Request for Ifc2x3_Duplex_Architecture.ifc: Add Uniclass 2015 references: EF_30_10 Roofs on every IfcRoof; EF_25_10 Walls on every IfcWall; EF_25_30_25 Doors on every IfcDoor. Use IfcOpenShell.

First a look at what the model holds.

```python
import ifcopenshell

model = ifcopenshell.open("Ifc2x3_Duplex_Architecture.ifc")
print(model.schema)
print("classifications:", [c.Name for c in model.by_type("IfcClassification")])
for ifc_class in ("IfcDoor", "IfcRoof", "IfcStair", "IfcWall", "IfcWindow"):
    print(ifc_class, len(model.by_type(ifc_class)))
```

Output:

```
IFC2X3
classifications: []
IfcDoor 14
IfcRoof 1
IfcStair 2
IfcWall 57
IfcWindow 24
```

```python
import ifcopenshell
import ifcopenshell.api.classification

model = ifcopenshell.open("Ifc2x3_Duplex_Architecture.ifc")

# IFC2X3 requires Source and Edition and has no link from the project to the system.
system = model.create_entity("IfcClassification", Source="NBS", Edition="2015", Name="Uniclass 2015")

codes = {
    "IfcRoof": ("EF_30_10", "Roofs"),
    "IfcWall": ("EF_25_10", "Walls"),
    "IfcDoor": ("EF_25_30_25", "Doors"),
}
for ifc_class, (code, name) in codes.items():
    products = model.by_type(ifc_class)
    ifcopenshell.api.classification.add_reference(
        model, products=products, classification=system, identification=code, name=name
    )
    print(code, len(products))

model.write("Ifc2x3_Duplex_Architecture_v2.ifc")
```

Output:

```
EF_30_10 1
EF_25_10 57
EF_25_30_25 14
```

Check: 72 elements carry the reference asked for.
